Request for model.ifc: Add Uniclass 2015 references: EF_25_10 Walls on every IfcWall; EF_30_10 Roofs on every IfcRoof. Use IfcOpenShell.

First a look at what the model holds.

```python
import ifcopenshell

model = ifcopenshell.open("model.ifc")
print(model.schema)
print("classifications:", [c.Name for c in model.by_type("IfcClassification")])
for ifc_class in ("IfcDoor", "IfcRoof", "IfcStair", "IfcWall", "IfcWindow"):
    print(ifc_class, len(model.by_type(ifc_class)))
```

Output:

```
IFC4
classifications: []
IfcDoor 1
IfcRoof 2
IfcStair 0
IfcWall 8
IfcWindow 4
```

```python
import ifcopenshell
import ifcopenshell.api.classification

model = ifcopenshell.open("model.ifc")

system = ifcopenshell.api.classification.add_classification(model, classification="Uniclass 2015")

codes = {
    "IfcWall": ("EF_25_10", "Walls"),
    "IfcRoof": ("EF_30_10", "Roofs"),
}
for ifc_class, (code, name) in codes.items():
    products = model.by_type(ifc_class)
    ifcopenshell.api.classification.add_reference(
        model, products=products, classification=system, identification=code, name=name
    )
    print(code, len(products))

model.write("model_updated.ifc")
```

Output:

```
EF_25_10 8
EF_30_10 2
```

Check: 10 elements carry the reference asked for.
